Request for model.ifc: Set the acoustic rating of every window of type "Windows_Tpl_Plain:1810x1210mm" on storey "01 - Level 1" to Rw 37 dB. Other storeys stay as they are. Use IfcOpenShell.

First a look at what the model holds.

```python
import ifcopenshell
import ifcopenshell.util.element

model = ifcopenshell.open("model.ifc")
print(model.schema)
storey = next(s for s in model.by_type("IfcBuildingStorey") if s.Name == "01 - Level 1")
windows = [e for e in ifcopenshell.util.element.get_decomposition(storey) if e.is_a("IfcWindow")]
seen = {}
for e in windows:
    element_type = ifcopenshell.util.element.get_type(e)
    key = (element_type.Name if element_type != e and element_type else None, ifcopenshell.util.element.get_pset(e, "Pset_WindowCommon", "AcousticRating"))
    seen[key] = seen.get(key, 0) + 1
for (name, value), count in sorted(seen.items(), key=str):
    print(count, "x", name, "|", value)
```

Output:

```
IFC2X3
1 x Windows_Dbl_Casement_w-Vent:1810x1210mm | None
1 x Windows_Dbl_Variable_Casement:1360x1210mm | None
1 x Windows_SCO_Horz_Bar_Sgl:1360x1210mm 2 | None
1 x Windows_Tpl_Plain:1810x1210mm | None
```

```python
import ifcopenshell
import ifcopenshell.api.pset
import ifcopenshell.util.element

model = ifcopenshell.open("model.ifc")

storey = next(s for s in model.by_type("IfcBuildingStorey") if s.Name == "01 - Level 1")
windows = [e for e in ifcopenshell.util.element.get_decomposition(storey) if e.is_a("IfcWindow")]

count = 0
for e in windows:
    element_type = ifcopenshell.util.element.get_type(e)
    if element_type in (None, e) or element_type.Name != "Windows_Tpl_Plain:1810x1210mm":
        continue
    # add_pset returns the element's existing set when there is one.
    pset = ifcopenshell.api.pset.add_pset(model, product=e, name="Pset_WindowCommon")
    ifcopenshell.api.pset.edit_pset(model, pset=pset, properties={"AcousticRating": "Rw 37 dB"})
    count += 1

print(count, "windows updated")

model.write("model_edited.ifc")
```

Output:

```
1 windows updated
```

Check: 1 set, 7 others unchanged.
